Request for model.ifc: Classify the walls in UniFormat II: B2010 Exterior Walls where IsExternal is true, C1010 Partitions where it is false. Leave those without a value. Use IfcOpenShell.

First a look at what the model holds.

```python
import ifcopenshell
import ifcopenshell.util.element

model = ifcopenshell.open("model.ifc")
print(model.schema)
print("classifications:", [c.Name for c in model.by_type("IfcClassification")])
values = [ifcopenshell.util.element.get_pset(e, "Pset_WallCommon", "IsExternal") for e in model.by_type("IfcWall")]
for value in (True, False, None):
    print("IsExternal", value, values.count(value))
```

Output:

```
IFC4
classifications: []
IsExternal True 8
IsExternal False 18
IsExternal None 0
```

```python
import ifcopenshell
import ifcopenshell.api.classification
import ifcopenshell.util.element

model = ifcopenshell.open("model.ifc")

system = ifcopenshell.api.classification.add_classification(model, classification="UniFormat II")

walls = model.by_type("IfcWall")
external = {e: ifcopenshell.util.element.get_pset(e, "Pset_WallCommon", "IsExternal") for e in walls}
for flag, code, name in ((True, "B2010", "Exterior Walls"), (False, "C1010", "Partitions")):
    products = [e for e in walls if external[e] is flag]
    ifcopenshell.api.classification.add_reference(
        model, products=products, classification=system, identification=code, name=name
    )
    print(code, len(products))

model.write("model_rev.ifc")
```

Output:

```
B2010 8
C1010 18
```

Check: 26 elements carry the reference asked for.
